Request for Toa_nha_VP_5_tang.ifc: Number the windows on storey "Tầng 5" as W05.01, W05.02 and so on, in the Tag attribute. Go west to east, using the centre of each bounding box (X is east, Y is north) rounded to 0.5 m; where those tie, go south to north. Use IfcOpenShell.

First a look at what the model holds.

```python
import ifcopenshell
import ifcopenshell.util.element
import ifcopenshell.util.placement

model = ifcopenshell.open("Toa_nha_VP_5_tang.ifc")
print(model.schema)
storey = next(s for s in model.by_type("IfcBuildingStorey") if s.Name == "Tầng 5")
windows = [e for e in ifcopenshell.util.element.get_decomposition(storey) if e.is_a("IfcWindow")]
for e in sorted(windows, key=lambda e: e.id()):
    origin = ifcopenshell.util.placement.get_local_placement(e.ObjectPlacement)[:3, 3]
    print(e.id(), e.Tag, e.Name, origin.round(2) + 0.0, sep=" | ")
```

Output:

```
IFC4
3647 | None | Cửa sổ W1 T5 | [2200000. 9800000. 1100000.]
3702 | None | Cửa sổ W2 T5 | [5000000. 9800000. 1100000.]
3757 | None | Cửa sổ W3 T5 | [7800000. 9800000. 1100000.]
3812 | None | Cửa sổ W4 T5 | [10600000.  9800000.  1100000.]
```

```python
import ifcopenshell
import ifcopenshell.geom
import ifcopenshell.util.element
import ifcopenshell.util.shape

model = ifcopenshell.open("Toa_nha_VP_5_tang.ifc")
settings = ifcopenshell.geom.settings()
settings.set("use-world-coords", True)


def centre(element):
    shape = ifcopenshell.geom.create_shape(settings, element)
    return ifcopenshell.util.shape.get_bbox_centroid(shape.geometry)


storey = next(s for s in model.by_type("IfcBuildingStorey") if s.Name == "Tầng 5")
windows = [e for e in ifcopenshell.util.element.get_decomposition(storey) if e.is_a("IfcWindow")]

# Insertion points can sit at a corner or the storey origin, so sort by the geometry (in metres).
centres = {e: centre(e) for e in windows}
windows.sort(key=lambda e: (round(centres[e][0] / 0.5), centres[e][1]))

for i, e in enumerate(windows, start=1):
    number = f"W05.{i:02d}"
    e.Tag = number
    print(e.id(), number)

model.write("Toa_nha_VP_5_tang-out.ifc")
```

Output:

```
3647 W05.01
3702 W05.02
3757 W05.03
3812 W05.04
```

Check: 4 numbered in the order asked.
